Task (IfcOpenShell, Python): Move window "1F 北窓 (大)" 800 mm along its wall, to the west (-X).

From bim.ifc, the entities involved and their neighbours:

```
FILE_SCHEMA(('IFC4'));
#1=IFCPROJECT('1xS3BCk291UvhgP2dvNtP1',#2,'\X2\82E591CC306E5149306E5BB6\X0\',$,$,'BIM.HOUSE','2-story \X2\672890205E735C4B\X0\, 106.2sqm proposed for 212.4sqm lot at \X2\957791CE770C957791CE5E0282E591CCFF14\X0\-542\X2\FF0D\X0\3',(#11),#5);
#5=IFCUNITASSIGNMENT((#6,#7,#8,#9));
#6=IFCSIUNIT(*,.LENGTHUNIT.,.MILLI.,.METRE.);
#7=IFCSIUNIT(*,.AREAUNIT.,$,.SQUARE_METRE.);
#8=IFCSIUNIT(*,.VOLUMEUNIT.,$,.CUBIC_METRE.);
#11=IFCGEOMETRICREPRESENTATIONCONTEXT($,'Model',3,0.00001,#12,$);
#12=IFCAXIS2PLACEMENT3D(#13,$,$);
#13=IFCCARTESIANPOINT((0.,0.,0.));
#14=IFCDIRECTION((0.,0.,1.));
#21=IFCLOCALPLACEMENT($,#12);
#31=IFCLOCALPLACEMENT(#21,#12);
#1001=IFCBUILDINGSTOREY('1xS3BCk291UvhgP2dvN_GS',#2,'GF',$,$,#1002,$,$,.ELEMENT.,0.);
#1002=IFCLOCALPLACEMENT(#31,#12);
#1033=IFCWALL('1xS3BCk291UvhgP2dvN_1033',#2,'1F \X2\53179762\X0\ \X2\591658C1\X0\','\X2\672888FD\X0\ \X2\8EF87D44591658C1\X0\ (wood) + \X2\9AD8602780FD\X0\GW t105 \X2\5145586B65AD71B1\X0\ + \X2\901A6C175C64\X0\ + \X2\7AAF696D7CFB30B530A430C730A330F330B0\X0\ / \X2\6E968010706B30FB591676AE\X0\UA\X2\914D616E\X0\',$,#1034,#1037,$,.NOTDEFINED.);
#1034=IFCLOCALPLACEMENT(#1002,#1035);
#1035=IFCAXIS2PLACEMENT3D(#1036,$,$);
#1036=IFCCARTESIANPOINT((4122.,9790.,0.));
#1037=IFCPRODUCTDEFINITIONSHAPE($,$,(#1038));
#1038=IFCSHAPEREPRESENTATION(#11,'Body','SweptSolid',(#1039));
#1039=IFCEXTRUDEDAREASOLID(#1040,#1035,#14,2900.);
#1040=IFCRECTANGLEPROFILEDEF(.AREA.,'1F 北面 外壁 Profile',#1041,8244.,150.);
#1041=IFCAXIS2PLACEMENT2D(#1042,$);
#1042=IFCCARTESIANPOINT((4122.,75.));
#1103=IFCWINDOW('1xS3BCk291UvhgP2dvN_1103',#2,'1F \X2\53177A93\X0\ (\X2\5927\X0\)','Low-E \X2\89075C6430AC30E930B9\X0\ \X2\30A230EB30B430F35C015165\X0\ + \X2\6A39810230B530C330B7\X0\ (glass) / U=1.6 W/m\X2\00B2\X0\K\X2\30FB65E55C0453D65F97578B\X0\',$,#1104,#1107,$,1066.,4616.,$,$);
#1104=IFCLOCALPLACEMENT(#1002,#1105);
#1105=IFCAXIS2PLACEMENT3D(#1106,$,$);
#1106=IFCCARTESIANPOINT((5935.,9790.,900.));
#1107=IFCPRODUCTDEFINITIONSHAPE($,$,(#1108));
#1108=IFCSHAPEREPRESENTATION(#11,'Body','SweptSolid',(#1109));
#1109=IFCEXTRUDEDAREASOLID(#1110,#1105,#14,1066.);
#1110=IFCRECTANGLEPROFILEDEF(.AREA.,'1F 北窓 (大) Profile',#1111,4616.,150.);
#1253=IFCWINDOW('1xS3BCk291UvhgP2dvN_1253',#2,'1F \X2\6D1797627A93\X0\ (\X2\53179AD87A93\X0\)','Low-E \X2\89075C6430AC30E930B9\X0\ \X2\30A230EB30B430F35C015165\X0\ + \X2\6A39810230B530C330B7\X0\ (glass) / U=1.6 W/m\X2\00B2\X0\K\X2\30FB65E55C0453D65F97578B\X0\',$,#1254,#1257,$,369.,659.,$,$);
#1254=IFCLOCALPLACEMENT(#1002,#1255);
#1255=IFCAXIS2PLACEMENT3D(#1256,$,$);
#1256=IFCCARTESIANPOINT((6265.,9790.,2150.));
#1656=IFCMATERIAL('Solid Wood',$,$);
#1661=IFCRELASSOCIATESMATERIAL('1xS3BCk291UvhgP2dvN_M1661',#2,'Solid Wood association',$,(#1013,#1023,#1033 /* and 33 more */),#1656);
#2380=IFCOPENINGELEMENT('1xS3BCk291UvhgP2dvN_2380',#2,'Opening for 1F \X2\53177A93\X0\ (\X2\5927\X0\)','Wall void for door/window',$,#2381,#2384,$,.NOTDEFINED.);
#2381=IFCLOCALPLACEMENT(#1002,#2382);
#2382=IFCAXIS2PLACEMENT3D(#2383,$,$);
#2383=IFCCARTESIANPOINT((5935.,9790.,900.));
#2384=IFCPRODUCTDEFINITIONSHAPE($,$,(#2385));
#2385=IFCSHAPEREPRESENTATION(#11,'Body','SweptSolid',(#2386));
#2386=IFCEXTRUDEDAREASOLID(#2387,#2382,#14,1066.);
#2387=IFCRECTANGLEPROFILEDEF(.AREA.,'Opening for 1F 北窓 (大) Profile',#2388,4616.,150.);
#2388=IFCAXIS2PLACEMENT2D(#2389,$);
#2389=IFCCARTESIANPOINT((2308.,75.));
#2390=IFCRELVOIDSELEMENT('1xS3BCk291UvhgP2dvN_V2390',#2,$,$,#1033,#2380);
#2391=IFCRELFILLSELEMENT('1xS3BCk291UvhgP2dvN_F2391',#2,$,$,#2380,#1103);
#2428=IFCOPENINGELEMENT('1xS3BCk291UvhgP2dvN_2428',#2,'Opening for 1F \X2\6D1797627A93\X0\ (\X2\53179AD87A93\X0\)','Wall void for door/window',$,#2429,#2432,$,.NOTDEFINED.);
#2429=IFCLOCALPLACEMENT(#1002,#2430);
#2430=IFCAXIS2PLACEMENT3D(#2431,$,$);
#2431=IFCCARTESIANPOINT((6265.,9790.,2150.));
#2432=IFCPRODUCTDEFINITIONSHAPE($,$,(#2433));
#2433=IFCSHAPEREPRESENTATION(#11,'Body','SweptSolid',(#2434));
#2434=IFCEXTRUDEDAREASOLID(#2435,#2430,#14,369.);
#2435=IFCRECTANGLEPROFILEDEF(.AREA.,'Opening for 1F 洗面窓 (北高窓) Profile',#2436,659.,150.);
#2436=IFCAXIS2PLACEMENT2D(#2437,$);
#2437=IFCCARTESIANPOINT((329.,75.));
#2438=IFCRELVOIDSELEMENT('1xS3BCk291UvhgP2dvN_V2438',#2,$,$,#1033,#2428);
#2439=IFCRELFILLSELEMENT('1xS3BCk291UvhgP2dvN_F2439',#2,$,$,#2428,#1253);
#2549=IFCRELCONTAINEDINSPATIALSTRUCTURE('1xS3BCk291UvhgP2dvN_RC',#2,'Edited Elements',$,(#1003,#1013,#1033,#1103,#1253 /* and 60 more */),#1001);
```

```python
import ifcopenshell
import ifcopenshell.api.geometry
import ifcopenshell.util.placement
import ifcopenshell.util.unit

model = ifcopenshell.open("bim.ifc")
unit_scale = ifcopenshell.util.unit.calculate_unit_scale(model)

window = model.by_guid("1xS3BCk291UvhgP2dvN_1103")
opening = window.FillsVoids[0].RelatingOpeningElement
wall = opening.VoidsElements[0].RelatingBuildingElement

wall_matrix = ifcopenshell.util.placement.get_local_placement(wall.ObjectPlacement)
shift = wall_matrix[:3, 0] * -0.8 / unit_scale
before = ifcopenshell.util.placement.get_local_placement(window.ObjectPlacement)[:3, 3].copy()

# The window is not placed relative to its opening, so move both.
for product in (opening, window):
    matrix = ifcopenshell.util.placement.get_local_placement(product.ObjectPlacement)
    matrix[:3, 3] += shift
    ifcopenshell.api.geometry.edit_object_placement(model, product=product, matrix=matrix, is_si=False)

after = ifcopenshell.util.placement.get_local_placement(window.ObjectPlacement)[:3, 3]
print("window moved by", (after - before).round(3) + 0.0)

model.write("bim_rev.ifc")
```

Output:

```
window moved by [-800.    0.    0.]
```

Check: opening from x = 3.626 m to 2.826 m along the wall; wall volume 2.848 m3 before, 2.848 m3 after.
